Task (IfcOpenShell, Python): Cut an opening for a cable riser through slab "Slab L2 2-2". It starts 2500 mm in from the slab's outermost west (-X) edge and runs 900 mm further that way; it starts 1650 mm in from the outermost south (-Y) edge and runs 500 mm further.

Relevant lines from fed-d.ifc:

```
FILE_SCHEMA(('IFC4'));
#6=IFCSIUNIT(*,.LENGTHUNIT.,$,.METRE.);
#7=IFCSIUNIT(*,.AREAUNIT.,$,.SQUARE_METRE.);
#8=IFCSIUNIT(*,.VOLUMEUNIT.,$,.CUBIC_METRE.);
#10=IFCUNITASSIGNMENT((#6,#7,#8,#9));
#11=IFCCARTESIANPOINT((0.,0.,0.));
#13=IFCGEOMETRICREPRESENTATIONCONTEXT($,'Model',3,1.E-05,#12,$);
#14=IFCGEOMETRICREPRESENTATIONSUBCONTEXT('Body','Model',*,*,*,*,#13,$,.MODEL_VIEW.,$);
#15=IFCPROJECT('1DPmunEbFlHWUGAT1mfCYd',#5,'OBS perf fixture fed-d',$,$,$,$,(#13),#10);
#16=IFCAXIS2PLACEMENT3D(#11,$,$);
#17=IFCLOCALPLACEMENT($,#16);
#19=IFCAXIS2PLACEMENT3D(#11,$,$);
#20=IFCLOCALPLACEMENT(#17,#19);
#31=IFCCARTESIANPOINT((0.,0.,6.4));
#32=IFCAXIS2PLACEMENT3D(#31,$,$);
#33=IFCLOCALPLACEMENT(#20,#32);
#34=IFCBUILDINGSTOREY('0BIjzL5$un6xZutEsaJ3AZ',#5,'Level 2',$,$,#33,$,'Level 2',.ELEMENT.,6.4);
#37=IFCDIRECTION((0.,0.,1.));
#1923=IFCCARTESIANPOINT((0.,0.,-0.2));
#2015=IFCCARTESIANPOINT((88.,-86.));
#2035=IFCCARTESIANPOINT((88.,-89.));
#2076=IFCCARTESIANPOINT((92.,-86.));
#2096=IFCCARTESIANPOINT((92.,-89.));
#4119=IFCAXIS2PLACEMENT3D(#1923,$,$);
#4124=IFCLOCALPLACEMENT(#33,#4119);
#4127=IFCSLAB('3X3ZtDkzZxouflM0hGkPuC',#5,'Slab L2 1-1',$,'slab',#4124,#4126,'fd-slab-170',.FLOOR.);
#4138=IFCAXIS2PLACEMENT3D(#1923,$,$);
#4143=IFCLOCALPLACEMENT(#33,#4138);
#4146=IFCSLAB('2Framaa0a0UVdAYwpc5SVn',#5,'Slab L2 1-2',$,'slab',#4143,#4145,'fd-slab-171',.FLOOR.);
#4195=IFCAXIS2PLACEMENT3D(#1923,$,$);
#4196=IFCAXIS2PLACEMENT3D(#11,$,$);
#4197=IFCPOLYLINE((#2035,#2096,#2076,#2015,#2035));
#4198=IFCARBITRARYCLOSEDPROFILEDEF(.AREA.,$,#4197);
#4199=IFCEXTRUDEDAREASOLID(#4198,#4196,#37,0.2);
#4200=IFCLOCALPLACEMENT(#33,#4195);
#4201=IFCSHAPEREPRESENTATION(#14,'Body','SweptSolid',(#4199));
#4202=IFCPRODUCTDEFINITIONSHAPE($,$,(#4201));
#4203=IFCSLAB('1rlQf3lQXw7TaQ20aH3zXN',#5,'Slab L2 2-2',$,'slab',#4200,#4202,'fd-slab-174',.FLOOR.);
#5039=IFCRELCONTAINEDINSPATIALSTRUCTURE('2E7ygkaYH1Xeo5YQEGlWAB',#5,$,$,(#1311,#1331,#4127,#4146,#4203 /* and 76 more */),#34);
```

```python
import numpy as np
import ifcopenshell
import ifcopenshell.api.feature
import ifcopenshell.api.geometry
import ifcopenshell.api.root
import ifcopenshell.geom
import ifcopenshell.util.placement
import ifcopenshell.util.representation
import ifcopenshell.util.shape
import ifcopenshell.util.unit

model = ifcopenshell.open("fed-d.ifc")
unit_scale = ifcopenshell.util.unit.calculate_unit_scale(model)
settings = ifcopenshell.geom.settings()


def volume(element):
    """Net volume in cubic metres, openings subtracted."""
    shape = ifcopenshell.geom.create_shape(settings, element)
    return ifcopenshell.util.shape.get_volume(shape.geometry)


slab = model.by_guid("1rlQf3lQXw7TaQ20aH3zXN")
before = volume(slab)

# Extent in the slab's own axes, in metres. The edges named are its -X and -Y sides.
slab_shape = ifcopenshell.geom.create_shape(settings, slab)
vertices = ifcopenshell.util.shape.get_vertices(slab_shape.geometry)
x_min, y_min, bottom = vertices.min(axis=0)
top = vertices[:, 2].max()

opening = ifcopenshell.api.root.create_entity(model, ifc_class="IfcOpeningElement", name="Cable riser opening", predefined_type="OPENING")
context = ifcopenshell.util.representation.get_context(model, "Model", "Body", "MODEL_VIEW")
width, depth = 0.9, 0.5
outline = [(0.0, 0.0), (width, 0.0), (width, depth), (0.0, depth), (0.0, 0.0)]
# Overshoot both faces by 50 mm so the cut is clean.
shape = ifcopenshell.api.geometry.add_slab_representation(
    model, context=context, depth=top - bottom + 0.1, polyline=outline
)
ifcopenshell.api.geometry.assign_representation(model, product=opening, representation=shape)

matrix = ifcopenshell.util.placement.get_local_placement(slab.ObjectPlacement)
matrix[:, 3] = matrix @ np.append(np.array([x_min + 2.5, y_min + 1.65, bottom - 0.05]) / unit_scale, 1.0)
ifcopenshell.api.geometry.edit_object_placement(model, product=opening, matrix=matrix, is_si=False)
ifcopenshell.api.feature.add_feature(model, feature=opening, element=slab)

after = volume(slab)

print(f"slab volume {before:.3f} -> {after:.3f} m3")

model.write("fed-d_rev.ifc")
```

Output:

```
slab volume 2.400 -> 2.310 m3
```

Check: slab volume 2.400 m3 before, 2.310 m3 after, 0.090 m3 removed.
